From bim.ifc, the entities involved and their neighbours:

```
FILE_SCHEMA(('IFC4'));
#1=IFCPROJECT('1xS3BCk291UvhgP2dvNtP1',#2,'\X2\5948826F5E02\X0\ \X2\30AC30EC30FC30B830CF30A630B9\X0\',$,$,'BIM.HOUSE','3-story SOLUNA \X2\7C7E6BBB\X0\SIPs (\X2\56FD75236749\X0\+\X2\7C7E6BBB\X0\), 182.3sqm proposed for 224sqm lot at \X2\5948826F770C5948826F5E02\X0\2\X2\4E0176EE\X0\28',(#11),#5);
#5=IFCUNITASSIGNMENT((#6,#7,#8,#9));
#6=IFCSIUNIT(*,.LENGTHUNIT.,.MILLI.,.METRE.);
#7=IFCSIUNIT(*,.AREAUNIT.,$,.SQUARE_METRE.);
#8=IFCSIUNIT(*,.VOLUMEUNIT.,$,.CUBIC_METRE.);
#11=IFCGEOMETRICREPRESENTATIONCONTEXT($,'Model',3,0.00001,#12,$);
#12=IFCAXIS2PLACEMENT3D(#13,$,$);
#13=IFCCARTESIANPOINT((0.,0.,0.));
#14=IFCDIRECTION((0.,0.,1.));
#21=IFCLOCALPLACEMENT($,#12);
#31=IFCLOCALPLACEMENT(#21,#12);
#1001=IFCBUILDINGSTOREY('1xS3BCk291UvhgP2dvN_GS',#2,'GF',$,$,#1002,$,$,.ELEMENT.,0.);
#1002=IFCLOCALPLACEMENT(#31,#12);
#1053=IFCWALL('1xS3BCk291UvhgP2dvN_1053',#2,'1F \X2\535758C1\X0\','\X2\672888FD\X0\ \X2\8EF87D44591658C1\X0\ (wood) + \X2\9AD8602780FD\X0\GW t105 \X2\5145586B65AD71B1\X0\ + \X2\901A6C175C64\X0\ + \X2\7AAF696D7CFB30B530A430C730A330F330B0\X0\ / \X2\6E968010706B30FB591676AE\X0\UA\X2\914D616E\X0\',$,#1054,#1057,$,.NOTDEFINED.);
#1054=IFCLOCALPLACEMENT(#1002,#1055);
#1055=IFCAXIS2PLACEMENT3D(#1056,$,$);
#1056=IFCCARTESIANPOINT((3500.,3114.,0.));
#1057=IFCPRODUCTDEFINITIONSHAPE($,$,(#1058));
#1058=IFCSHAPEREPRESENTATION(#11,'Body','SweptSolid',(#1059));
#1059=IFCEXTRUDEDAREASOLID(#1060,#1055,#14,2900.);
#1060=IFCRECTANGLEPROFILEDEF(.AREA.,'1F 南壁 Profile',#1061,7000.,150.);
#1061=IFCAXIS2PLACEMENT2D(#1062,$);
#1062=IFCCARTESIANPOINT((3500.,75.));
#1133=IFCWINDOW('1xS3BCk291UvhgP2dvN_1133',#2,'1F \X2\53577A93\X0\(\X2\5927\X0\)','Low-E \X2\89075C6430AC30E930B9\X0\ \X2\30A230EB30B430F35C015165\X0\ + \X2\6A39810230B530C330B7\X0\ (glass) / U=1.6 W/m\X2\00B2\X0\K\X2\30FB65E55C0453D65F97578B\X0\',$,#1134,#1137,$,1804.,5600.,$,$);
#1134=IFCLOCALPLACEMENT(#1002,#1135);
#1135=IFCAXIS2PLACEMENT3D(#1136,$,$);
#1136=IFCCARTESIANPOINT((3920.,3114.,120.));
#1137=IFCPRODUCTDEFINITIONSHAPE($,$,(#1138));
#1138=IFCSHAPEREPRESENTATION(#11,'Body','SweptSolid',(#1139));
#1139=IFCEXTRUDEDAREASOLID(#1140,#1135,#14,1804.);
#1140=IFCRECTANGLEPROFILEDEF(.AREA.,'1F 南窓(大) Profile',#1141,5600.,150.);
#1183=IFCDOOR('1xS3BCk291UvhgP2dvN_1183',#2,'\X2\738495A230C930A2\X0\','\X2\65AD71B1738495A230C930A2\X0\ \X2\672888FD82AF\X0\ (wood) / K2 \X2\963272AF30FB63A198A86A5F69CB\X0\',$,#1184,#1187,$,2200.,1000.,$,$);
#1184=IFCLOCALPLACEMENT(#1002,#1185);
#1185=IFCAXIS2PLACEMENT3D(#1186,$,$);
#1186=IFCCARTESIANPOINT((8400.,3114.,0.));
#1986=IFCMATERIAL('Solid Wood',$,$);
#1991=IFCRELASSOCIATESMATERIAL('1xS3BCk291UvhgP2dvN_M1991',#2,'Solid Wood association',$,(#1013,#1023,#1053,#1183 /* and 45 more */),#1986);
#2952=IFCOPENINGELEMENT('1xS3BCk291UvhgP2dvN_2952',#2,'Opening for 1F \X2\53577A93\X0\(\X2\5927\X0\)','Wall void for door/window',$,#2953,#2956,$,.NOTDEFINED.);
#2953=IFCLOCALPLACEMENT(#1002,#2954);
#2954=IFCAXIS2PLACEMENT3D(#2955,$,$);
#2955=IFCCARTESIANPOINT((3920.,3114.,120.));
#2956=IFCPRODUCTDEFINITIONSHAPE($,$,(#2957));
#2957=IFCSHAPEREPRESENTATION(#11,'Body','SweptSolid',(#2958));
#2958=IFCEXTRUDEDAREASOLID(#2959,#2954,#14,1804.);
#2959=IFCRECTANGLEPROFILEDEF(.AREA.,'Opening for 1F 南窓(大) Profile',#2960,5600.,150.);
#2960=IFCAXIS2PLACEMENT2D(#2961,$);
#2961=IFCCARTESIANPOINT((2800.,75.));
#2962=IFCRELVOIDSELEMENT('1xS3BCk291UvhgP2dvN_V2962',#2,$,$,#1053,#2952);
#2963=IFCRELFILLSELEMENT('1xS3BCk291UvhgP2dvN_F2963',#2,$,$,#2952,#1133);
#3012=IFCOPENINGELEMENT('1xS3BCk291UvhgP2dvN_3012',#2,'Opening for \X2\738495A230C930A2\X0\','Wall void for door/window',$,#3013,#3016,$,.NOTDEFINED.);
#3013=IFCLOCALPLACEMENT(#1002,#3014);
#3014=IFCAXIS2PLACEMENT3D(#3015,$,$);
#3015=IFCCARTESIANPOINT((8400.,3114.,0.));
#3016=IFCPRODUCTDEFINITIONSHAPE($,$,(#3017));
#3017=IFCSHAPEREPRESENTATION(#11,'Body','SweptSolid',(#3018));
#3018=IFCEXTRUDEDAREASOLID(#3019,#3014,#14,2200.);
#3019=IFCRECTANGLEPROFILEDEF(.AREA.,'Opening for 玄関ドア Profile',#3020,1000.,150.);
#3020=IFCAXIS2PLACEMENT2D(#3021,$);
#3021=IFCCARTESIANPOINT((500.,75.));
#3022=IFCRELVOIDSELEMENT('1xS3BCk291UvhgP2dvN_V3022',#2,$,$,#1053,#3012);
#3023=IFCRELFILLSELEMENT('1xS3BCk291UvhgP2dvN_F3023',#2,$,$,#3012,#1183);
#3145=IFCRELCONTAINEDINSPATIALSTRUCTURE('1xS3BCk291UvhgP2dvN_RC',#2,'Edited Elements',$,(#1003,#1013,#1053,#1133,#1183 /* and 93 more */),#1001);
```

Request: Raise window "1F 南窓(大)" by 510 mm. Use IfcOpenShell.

```python
import numpy as np
import ifcopenshell
import ifcopenshell.api.geometry
import ifcopenshell.util.placement
import ifcopenshell.util.unit

model = ifcopenshell.open("bim.ifc")
unit_scale = ifcopenshell.util.unit.calculate_unit_scale(model)

window = model.by_id(1133)
opening = window.FillsVoids[0].RelatingOpeningElement
dz = 510.0

shift = np.array([0.0, 0.0, dz])
# The window is not placed relative to its opening, so move both.
for product in (opening, window):
    matrix = ifcopenshell.util.placement.get_local_placement(product.ObjectPlacement)
    matrix[:3, 3] += shift
    ifcopenshell.api.geometry.edit_object_placement(model, product=product, matrix=matrix, is_si=False)

print(f"moved by {dz * unit_scale:+.3f} m")

model.write("bim_rev.ifc")
```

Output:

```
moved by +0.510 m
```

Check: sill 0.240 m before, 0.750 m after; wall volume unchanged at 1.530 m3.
